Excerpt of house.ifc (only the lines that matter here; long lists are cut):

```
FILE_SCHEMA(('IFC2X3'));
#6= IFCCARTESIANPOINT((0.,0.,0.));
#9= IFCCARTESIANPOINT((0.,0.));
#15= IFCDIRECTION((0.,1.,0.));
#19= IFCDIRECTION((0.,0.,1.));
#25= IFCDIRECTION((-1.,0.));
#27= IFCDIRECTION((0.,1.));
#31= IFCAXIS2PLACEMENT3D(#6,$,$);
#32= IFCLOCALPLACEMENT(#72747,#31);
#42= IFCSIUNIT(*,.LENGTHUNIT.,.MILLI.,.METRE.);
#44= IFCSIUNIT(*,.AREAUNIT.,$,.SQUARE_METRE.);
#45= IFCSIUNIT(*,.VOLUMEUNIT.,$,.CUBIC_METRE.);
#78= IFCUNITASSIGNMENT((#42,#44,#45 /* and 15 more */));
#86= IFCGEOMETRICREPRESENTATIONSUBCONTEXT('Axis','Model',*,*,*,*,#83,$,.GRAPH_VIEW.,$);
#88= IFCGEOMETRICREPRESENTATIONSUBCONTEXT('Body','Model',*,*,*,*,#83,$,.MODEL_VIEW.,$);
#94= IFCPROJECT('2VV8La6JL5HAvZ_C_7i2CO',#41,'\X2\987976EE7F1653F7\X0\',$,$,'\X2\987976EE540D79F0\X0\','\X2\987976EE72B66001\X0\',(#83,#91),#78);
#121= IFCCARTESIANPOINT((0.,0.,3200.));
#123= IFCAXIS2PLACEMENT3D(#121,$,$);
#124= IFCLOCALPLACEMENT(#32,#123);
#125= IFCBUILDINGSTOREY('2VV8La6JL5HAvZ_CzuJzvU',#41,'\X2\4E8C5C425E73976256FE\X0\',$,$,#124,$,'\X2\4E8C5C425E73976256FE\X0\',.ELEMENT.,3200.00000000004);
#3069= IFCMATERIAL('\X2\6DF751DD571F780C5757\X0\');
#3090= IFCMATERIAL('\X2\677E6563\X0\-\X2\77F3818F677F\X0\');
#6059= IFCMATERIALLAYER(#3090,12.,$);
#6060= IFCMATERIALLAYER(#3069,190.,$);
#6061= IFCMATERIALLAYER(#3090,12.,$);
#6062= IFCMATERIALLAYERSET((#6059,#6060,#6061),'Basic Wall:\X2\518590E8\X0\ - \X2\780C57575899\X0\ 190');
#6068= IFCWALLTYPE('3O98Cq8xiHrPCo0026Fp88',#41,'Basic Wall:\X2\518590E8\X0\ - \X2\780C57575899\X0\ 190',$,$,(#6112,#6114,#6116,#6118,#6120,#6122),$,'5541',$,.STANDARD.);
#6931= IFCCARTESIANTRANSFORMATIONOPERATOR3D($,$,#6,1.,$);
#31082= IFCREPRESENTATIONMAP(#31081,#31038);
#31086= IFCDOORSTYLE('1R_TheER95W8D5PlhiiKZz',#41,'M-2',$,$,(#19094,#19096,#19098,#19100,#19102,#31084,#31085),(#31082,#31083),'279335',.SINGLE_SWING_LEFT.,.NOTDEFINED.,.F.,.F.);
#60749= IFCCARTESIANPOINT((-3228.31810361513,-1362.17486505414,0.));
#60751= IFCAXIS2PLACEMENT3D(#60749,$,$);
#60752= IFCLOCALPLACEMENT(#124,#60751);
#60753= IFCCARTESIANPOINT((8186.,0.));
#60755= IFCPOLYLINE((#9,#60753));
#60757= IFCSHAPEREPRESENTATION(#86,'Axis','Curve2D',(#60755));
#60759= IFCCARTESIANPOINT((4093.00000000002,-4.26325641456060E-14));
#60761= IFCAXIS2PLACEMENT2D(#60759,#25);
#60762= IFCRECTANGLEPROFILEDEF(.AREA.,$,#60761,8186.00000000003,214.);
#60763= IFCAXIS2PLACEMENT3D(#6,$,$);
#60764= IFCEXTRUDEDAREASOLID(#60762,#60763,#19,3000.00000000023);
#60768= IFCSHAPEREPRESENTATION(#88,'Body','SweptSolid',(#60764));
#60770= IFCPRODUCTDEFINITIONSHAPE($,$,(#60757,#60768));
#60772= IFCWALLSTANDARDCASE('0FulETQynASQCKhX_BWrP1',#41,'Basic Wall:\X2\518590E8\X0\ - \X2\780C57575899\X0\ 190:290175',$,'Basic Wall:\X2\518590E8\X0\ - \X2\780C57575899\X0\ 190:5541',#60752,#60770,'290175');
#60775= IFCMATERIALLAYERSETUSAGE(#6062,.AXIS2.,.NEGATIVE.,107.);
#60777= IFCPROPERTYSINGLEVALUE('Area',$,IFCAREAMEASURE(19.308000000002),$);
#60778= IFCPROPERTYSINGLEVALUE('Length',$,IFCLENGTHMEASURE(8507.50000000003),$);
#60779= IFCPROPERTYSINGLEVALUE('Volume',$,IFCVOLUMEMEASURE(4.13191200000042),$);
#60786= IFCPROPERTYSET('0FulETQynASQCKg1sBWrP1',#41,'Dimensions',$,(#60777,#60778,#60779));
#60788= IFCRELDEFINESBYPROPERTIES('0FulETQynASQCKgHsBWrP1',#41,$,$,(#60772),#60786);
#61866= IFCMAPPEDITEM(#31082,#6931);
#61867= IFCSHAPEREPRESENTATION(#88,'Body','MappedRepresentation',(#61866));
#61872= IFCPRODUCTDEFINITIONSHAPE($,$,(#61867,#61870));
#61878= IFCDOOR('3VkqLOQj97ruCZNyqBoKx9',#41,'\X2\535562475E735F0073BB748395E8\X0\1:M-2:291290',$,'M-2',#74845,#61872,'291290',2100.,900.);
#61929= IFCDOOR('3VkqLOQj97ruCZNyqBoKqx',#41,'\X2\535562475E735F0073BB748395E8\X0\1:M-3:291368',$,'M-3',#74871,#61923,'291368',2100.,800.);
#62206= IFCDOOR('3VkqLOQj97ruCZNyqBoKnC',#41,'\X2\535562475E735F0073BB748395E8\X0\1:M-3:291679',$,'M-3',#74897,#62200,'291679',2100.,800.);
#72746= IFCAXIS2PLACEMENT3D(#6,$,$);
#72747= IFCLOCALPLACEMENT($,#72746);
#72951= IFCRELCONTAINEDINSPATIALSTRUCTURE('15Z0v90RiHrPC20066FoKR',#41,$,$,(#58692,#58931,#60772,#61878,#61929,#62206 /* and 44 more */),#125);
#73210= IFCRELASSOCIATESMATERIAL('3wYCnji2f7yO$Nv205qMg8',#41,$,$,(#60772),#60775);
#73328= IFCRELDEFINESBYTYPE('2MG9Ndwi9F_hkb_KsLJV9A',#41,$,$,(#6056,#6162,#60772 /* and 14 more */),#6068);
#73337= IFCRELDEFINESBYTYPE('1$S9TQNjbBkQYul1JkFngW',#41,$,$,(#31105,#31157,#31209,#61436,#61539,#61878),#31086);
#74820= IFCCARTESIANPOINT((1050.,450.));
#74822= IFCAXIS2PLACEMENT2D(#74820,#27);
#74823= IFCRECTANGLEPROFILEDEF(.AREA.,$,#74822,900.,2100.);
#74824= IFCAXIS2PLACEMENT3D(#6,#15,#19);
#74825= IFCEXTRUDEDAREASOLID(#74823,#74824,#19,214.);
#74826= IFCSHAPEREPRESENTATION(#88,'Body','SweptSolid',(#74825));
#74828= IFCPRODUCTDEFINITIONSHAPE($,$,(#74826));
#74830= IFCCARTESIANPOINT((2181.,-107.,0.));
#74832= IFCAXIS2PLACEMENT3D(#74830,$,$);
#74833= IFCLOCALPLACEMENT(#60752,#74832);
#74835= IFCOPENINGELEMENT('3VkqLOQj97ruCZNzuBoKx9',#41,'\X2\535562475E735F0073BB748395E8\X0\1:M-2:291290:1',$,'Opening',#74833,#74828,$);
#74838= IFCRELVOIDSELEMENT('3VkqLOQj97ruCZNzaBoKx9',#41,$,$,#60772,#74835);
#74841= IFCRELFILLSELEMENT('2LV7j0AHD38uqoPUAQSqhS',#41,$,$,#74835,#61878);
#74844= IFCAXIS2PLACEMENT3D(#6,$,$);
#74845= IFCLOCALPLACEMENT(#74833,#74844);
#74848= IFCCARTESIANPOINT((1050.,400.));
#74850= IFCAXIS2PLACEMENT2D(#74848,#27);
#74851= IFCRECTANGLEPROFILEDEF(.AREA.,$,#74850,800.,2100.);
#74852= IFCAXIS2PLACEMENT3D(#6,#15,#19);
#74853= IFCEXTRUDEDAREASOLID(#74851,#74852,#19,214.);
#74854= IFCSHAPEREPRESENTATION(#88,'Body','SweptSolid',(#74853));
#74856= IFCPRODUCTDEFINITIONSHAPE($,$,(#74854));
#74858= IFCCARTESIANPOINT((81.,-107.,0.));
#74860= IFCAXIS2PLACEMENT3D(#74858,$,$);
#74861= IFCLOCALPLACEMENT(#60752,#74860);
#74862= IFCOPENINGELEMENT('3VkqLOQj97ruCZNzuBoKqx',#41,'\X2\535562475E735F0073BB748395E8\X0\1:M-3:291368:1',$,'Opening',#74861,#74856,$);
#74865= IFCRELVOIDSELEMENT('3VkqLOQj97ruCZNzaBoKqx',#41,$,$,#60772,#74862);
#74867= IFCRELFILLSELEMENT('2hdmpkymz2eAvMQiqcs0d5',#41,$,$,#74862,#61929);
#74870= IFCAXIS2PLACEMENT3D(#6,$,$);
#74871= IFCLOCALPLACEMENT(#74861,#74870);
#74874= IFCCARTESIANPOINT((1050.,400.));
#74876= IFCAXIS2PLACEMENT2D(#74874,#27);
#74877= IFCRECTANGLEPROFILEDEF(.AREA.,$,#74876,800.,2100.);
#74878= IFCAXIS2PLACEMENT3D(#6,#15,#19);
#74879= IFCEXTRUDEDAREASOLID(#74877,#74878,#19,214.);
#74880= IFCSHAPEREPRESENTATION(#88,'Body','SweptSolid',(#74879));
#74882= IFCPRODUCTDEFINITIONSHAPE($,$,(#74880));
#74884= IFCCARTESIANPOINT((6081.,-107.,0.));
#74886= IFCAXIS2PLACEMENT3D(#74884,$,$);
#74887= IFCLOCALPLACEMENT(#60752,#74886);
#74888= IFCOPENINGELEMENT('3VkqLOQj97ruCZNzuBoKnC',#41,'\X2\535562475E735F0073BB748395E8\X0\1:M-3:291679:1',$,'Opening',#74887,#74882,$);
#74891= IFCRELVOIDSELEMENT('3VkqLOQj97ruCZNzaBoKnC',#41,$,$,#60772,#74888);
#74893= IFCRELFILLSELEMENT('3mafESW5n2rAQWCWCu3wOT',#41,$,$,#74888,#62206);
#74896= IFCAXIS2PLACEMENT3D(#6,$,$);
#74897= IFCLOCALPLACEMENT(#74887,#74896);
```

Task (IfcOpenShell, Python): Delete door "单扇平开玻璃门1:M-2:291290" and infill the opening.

```python
import ifcopenshell
import ifcopenshell.api.feature
import ifcopenshell.api.pset
import ifcopenshell.api.root
import ifcopenshell.geom
import ifcopenshell.util.element
import ifcopenshell.util.shape
import ifcopenshell.util.unit

model = ifcopenshell.open("house.ifc")
area_scale = ifcopenshell.util.unit.calculate_unit_scale(model, "AREAUNIT")
volume_scale = ifcopenshell.util.unit.calculate_unit_scale(model, "VOLUMEUNIT")
settings = ifcopenshell.geom.settings()


def volume(element):
    """Net volume in cubic metres, openings subtracted."""
    shape = ifcopenshell.geom.create_shape(settings, element)
    return ifcopenshell.util.shape.get_volume(shape.geometry)


door = model.by_guid("3VkqLOQj97ruCZNyqBoKx9")
opening = door.FillsVoids[0].RelatingOpeningElement
wall = opening.VoidsElements[0].RelatingBuildingElement
before = volume(wall)

ifcopenshell.api.root.remove_product(model, product=door)
ifcopenshell.api.feature.remove_feature(model, feature=opening)

after = volume(wall)
thickness = 0.214  # wall thickness in metres

# Update the wall's stored quantities.
pset = model.by_id(ifcopenshell.util.element.get_pset(wall, "Dimensions", should_inherit=False)["id"])
ifcopenshell.api.pset.edit_pset(model, pset=pset, properties={
    "Area": model.create_entity("IfcAreaMeasure", after / thickness / area_scale),
    "Volume": model.create_entity("IfcVolumeMeasure", after / volume_scale),
})

print(f"wall volume {before:.3f} -> {after:.3f} m3")

model.write("house-out.ifc")
```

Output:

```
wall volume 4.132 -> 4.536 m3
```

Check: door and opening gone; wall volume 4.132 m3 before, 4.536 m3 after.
